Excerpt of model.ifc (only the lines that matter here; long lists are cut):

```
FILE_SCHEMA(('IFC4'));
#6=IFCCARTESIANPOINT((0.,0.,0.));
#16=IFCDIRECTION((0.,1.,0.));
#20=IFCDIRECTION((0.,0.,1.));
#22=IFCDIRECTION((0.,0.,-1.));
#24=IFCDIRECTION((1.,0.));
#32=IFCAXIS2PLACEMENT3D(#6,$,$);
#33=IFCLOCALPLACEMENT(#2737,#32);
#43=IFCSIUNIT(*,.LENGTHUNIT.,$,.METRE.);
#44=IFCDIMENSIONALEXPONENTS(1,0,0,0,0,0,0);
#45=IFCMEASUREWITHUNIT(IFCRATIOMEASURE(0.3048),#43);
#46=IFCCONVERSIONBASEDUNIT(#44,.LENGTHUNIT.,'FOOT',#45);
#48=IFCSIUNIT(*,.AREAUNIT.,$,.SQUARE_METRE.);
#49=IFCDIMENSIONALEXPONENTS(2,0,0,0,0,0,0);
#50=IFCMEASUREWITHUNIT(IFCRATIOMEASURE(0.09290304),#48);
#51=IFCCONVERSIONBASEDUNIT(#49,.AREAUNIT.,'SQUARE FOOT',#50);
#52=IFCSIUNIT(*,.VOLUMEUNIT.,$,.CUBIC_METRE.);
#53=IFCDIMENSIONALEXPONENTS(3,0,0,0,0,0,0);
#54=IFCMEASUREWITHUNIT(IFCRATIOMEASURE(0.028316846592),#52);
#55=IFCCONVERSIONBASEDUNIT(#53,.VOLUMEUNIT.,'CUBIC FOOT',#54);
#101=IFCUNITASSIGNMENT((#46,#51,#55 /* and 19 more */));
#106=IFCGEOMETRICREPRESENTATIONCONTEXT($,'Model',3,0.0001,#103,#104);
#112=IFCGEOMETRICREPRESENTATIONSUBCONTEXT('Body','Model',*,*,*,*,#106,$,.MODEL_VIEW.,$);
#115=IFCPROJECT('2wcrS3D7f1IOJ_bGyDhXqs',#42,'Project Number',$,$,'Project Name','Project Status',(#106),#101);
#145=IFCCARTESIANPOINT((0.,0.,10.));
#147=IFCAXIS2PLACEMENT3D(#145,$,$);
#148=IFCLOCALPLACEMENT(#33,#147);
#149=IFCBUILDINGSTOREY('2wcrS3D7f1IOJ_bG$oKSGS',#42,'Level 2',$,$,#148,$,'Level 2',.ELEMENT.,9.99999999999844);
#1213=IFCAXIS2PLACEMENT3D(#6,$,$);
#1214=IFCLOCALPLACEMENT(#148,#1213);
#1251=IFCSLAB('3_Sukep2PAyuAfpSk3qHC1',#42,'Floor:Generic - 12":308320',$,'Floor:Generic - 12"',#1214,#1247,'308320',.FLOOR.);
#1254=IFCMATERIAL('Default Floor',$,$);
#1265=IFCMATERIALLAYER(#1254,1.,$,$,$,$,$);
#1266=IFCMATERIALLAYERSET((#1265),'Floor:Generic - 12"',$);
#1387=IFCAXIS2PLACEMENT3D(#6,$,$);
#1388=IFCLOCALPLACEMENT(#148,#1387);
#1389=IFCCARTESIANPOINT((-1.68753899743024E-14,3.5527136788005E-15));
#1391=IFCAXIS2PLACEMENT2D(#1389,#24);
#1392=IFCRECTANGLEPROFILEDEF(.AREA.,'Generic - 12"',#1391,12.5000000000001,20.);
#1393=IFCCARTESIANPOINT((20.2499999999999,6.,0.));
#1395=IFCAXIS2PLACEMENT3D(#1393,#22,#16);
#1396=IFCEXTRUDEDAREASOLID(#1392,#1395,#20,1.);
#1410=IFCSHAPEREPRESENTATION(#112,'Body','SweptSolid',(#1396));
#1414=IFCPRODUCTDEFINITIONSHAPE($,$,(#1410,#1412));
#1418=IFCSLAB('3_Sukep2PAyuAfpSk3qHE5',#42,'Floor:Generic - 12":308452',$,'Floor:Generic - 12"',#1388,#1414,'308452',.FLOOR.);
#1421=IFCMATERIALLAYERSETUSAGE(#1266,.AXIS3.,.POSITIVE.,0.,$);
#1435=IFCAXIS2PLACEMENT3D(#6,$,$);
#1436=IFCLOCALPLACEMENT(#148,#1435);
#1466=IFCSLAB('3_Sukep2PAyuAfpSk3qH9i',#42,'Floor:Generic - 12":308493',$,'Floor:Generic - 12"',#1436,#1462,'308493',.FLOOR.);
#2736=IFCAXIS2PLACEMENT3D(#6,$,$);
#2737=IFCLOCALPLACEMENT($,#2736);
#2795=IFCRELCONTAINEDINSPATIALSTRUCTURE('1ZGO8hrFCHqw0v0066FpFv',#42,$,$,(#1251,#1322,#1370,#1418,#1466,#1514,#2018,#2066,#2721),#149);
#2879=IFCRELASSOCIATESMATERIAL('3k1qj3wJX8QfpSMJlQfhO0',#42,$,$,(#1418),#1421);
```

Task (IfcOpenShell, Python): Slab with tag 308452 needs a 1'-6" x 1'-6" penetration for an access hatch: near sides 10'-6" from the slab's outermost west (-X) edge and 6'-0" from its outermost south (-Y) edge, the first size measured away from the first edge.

```python
import numpy as np
import ifcopenshell
import ifcopenshell.api.feature
import ifcopenshell.api.geometry
import ifcopenshell.api.root
import ifcopenshell.geom
import ifcopenshell.util.placement
import ifcopenshell.util.representation
import ifcopenshell.util.shape
import ifcopenshell.util.unit

model = ifcopenshell.open("model.ifc")
unit_scale = ifcopenshell.util.unit.calculate_unit_scale(model)
settings = ifcopenshell.geom.settings()


def volume(element):
    """Net volume in cubic metres, openings subtracted."""
    shape = ifcopenshell.geom.create_shape(settings, element)
    return ifcopenshell.util.shape.get_volume(shape.geometry)


slab = model.by_guid("3_Sukep2PAyuAfpSk3qHE5")
before = volume(slab)

# Extent in the slab's own axes, in metres. The edges named are its -X and -Y sides.
slab_shape = ifcopenshell.geom.create_shape(settings, slab)
vertices = ifcopenshell.util.shape.get_vertices(slab_shape.geometry)
x_min, y_min, bottom = vertices.min(axis=0)
top = vertices[:, 2].max()

opening = ifcopenshell.api.root.create_entity(model, ifc_class="IfcOpeningElement", name="Access hatch opening", predefined_type="OPENING")
context = ifcopenshell.util.representation.get_context(model, "Model", "Body", "MODEL_VIEW")
width, depth = 0.4572, 0.4572
outline = [(0.0, 0.0), (width, 0.0), (width, depth), (0.0, depth), (0.0, 0.0)]
# Overshoot both faces by 50 mm so the cut is clean.
shape = ifcopenshell.api.geometry.add_slab_representation(
    model, context=context, depth=top - bottom + 0.1, polyline=outline
)
ifcopenshell.api.geometry.assign_representation(model, product=opening, representation=shape)

matrix = ifcopenshell.util.placement.get_local_placement(slab.ObjectPlacement)
matrix[:, 3] = matrix @ np.append(np.array([x_min + 3.2004, y_min + 1.8288, bottom - 0.05]) / unit_scale, 1.0)
ifcopenshell.api.geometry.edit_object_placement(model, product=opening, matrix=matrix, is_si=False)
ifcopenshell.api.feature.add_feature(model, feature=opening, element=slab)

after = volume(slab)

print(f"slab volume {before:.3f} -> {after:.3f} m3")

model.write("model_v2.ifc")
```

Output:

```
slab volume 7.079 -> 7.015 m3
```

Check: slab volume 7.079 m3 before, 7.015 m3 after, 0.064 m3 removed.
